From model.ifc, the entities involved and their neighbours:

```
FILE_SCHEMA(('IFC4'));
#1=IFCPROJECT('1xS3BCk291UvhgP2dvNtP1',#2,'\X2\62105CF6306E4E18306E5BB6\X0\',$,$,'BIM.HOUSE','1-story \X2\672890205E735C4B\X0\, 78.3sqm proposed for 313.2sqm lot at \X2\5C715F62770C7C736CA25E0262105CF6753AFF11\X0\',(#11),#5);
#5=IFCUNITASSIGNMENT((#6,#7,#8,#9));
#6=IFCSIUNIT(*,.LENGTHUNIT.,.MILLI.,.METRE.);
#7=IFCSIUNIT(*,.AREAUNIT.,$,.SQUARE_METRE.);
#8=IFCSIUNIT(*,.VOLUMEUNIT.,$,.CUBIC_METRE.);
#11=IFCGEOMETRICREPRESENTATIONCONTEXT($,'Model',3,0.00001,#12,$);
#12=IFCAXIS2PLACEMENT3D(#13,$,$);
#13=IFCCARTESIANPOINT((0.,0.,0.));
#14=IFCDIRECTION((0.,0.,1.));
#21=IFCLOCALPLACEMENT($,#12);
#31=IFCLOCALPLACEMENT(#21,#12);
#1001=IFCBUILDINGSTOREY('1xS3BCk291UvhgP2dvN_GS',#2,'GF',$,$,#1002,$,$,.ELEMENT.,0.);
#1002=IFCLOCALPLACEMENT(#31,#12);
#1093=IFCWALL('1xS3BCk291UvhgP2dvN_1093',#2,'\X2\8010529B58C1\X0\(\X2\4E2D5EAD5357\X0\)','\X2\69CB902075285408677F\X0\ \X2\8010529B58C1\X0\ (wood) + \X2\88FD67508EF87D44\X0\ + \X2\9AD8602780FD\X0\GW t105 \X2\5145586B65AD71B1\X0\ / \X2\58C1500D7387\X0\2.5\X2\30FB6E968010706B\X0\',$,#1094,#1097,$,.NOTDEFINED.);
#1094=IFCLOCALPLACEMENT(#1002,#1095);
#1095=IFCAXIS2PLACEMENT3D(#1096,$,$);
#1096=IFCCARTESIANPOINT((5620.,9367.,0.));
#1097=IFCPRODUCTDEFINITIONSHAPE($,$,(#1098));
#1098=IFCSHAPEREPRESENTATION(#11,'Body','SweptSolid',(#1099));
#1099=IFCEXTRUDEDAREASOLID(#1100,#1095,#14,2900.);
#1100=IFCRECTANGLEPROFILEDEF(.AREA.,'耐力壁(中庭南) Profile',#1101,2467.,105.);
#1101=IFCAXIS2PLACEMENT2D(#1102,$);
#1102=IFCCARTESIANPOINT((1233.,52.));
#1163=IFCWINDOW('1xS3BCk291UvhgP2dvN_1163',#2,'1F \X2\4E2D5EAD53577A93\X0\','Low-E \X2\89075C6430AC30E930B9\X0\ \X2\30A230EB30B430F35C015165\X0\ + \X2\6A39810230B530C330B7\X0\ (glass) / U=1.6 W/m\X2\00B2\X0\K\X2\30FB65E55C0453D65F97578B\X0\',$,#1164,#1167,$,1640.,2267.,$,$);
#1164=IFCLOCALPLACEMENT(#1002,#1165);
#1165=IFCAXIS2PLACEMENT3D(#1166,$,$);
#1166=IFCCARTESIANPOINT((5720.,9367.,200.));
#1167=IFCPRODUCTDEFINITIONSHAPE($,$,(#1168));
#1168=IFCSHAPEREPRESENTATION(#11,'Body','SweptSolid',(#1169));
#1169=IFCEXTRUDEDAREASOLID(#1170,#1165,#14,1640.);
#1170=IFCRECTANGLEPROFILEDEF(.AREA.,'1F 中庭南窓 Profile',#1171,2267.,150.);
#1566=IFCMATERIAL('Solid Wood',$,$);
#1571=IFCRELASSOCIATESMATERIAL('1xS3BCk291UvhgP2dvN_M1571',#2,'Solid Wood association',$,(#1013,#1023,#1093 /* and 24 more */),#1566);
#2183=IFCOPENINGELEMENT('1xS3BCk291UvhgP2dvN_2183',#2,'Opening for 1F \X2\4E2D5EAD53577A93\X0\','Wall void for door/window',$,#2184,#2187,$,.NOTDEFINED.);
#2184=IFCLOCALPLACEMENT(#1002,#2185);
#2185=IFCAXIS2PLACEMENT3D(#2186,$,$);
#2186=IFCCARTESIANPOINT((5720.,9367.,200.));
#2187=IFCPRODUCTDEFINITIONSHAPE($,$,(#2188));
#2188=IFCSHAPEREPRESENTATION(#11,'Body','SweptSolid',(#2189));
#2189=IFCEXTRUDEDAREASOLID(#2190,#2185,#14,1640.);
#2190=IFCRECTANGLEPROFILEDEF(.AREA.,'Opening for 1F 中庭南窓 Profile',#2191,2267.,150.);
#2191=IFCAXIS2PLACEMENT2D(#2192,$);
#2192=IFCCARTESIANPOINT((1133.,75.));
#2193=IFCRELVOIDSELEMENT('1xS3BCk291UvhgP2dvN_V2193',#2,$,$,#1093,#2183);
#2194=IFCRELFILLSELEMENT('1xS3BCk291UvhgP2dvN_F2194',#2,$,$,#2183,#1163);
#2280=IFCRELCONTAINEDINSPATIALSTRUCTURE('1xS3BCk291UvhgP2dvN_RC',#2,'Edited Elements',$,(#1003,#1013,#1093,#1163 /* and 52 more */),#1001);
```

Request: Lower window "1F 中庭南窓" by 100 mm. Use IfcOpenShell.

```python
import numpy as np
import ifcopenshell
import ifcopenshell.api.geometry
import ifcopenshell.util.placement
import ifcopenshell.util.unit

model = ifcopenshell.open("model.ifc")
unit_scale = ifcopenshell.util.unit.calculate_unit_scale(model)

window = model.by_guid("1xS3BCk291UvhgP2dvN_1163")
opening = window.FillsVoids[0].RelatingOpeningElement
dz = -100.0

shift = np.array([0.0, 0.0, dz])
# The window is not placed relative to its opening, so move both.
for product in (opening, window):
    matrix = ifcopenshell.util.placement.get_local_placement(product.ObjectPlacement)
    matrix[:3, 3] += shift
    ifcopenshell.api.geometry.edit_object_placement(model, product=product, matrix=matrix, is_si=False)

print(f"moved by {dz * unit_scale:+.3f} m")

model.write("model_v2.ifc")
```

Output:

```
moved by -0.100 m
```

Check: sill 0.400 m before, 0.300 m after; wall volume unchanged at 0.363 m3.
